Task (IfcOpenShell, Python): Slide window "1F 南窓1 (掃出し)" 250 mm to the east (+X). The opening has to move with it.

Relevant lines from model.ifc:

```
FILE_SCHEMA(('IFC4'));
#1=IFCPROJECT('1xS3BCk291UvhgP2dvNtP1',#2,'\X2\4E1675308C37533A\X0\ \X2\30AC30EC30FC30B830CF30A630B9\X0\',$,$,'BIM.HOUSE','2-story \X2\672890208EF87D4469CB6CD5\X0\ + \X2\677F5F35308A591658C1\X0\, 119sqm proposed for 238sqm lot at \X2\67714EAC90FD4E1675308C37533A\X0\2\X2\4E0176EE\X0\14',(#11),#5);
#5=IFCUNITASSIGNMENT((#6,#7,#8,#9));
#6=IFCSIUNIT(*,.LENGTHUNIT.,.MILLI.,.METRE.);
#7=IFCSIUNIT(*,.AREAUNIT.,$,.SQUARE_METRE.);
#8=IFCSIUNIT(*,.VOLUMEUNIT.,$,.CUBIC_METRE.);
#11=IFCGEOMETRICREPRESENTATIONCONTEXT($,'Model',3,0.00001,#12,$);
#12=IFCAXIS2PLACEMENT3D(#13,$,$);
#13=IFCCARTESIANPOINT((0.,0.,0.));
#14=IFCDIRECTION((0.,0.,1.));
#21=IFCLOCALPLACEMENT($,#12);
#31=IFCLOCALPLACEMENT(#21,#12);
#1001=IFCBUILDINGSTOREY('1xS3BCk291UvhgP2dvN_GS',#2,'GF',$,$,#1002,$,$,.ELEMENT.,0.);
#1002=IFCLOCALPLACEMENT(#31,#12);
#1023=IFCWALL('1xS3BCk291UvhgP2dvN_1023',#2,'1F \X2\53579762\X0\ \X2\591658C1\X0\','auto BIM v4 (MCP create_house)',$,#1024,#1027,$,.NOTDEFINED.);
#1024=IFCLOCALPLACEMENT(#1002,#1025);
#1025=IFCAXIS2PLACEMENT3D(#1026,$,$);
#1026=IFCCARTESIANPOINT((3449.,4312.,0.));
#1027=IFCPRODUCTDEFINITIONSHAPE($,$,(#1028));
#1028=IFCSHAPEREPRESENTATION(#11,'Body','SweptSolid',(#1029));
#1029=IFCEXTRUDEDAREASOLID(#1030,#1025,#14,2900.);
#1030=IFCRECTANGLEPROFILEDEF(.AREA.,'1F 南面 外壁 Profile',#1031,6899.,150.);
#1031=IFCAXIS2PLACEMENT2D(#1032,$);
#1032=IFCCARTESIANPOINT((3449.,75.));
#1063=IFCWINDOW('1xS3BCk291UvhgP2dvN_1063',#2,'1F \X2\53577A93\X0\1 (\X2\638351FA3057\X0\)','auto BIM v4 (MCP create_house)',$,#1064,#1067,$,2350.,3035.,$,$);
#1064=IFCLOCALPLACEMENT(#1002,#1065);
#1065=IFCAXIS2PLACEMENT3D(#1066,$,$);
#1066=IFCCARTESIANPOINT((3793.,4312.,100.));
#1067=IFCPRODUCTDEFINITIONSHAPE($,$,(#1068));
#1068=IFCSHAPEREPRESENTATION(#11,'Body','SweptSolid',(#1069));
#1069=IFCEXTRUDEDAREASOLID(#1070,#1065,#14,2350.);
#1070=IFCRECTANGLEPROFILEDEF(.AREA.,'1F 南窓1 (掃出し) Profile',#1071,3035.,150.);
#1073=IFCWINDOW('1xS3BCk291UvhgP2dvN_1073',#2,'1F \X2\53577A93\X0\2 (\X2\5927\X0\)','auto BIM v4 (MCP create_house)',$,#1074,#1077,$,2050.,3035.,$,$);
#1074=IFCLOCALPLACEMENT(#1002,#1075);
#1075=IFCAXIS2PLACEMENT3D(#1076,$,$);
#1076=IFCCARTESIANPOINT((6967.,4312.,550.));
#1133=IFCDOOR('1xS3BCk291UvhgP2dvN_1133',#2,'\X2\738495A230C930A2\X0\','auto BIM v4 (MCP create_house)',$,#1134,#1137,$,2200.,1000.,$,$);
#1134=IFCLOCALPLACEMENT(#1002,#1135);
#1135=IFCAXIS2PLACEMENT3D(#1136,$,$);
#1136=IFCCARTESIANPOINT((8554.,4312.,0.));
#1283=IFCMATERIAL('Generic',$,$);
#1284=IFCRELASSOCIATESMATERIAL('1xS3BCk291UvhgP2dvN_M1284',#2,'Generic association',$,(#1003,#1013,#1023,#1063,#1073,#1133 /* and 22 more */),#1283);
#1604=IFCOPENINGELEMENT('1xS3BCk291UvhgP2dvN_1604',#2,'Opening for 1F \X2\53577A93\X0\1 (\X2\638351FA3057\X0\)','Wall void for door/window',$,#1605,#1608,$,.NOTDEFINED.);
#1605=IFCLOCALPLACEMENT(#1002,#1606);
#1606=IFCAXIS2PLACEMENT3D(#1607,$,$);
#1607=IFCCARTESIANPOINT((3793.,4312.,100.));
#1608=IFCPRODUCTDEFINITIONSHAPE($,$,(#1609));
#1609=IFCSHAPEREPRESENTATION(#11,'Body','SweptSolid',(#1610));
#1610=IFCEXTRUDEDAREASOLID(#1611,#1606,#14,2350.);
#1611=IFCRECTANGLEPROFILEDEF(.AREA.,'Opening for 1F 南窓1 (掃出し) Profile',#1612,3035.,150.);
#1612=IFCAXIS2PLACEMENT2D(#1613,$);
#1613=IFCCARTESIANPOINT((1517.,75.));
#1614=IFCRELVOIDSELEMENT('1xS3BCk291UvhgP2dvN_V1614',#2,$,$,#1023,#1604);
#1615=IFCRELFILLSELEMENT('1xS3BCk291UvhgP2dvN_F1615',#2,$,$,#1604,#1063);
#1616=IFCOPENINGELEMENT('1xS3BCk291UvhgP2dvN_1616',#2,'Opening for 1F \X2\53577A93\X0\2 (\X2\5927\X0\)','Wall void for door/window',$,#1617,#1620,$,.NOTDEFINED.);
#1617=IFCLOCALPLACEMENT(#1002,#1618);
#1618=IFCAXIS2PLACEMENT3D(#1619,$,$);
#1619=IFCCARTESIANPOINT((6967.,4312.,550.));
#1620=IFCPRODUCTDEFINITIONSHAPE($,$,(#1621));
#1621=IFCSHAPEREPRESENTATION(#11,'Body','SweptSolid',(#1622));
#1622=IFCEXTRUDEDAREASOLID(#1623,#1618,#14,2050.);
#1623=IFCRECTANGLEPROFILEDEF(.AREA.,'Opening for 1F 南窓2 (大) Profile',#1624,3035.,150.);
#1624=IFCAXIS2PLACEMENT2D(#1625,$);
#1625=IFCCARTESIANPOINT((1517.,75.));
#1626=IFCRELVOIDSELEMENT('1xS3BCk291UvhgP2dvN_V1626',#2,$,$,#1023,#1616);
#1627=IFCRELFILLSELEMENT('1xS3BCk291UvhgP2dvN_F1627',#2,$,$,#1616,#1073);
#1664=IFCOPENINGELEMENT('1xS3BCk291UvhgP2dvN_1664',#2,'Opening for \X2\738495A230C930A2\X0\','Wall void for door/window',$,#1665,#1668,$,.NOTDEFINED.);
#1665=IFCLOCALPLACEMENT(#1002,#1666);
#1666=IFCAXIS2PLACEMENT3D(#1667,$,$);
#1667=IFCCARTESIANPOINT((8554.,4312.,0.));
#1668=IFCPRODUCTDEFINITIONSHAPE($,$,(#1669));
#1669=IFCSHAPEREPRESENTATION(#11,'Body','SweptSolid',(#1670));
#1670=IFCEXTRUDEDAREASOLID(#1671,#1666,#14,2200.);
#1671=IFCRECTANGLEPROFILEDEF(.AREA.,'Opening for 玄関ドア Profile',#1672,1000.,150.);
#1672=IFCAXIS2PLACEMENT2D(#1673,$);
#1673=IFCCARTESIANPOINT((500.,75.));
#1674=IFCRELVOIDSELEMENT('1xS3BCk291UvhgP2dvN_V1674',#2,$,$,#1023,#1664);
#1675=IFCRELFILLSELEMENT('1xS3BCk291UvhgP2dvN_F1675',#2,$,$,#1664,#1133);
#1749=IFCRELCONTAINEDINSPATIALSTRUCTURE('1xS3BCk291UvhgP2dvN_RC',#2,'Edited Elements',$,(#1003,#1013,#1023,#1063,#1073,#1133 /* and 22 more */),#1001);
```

```python
import ifcopenshell
import ifcopenshell.api.geometry
import ifcopenshell.util.placement
import ifcopenshell.util.unit

model = ifcopenshell.open("model.ifc")
unit_scale = ifcopenshell.util.unit.calculate_unit_scale(model)

window = model.by_id(1063)
opening = window.FillsVoids[0].RelatingOpeningElement
wall = opening.VoidsElements[0].RelatingBuildingElement

wall_matrix = ifcopenshell.util.placement.get_local_placement(wall.ObjectPlacement)
shift = wall_matrix[:3, 0] * 0.25 / unit_scale
before = ifcopenshell.util.placement.get_local_placement(window.ObjectPlacement)[:3, 3].copy()

# The window is not placed relative to its opening, so move both.
for product in (opening, window):
    matrix = ifcopenshell.util.placement.get_local_placement(product.ObjectPlacement)
    matrix[:3, 3] += shift
    ifcopenshell.api.geometry.edit_object_placement(model, product=product, matrix=matrix, is_si=False)

after = ifcopenshell.util.placement.get_local_placement(window.ObjectPlacement)[:3, 3]
print("window moved by", (after - before).round(3) + 0.0)

model.write("model_rev.ifc")
```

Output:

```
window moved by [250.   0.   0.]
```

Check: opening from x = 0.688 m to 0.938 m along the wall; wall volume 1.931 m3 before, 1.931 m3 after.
